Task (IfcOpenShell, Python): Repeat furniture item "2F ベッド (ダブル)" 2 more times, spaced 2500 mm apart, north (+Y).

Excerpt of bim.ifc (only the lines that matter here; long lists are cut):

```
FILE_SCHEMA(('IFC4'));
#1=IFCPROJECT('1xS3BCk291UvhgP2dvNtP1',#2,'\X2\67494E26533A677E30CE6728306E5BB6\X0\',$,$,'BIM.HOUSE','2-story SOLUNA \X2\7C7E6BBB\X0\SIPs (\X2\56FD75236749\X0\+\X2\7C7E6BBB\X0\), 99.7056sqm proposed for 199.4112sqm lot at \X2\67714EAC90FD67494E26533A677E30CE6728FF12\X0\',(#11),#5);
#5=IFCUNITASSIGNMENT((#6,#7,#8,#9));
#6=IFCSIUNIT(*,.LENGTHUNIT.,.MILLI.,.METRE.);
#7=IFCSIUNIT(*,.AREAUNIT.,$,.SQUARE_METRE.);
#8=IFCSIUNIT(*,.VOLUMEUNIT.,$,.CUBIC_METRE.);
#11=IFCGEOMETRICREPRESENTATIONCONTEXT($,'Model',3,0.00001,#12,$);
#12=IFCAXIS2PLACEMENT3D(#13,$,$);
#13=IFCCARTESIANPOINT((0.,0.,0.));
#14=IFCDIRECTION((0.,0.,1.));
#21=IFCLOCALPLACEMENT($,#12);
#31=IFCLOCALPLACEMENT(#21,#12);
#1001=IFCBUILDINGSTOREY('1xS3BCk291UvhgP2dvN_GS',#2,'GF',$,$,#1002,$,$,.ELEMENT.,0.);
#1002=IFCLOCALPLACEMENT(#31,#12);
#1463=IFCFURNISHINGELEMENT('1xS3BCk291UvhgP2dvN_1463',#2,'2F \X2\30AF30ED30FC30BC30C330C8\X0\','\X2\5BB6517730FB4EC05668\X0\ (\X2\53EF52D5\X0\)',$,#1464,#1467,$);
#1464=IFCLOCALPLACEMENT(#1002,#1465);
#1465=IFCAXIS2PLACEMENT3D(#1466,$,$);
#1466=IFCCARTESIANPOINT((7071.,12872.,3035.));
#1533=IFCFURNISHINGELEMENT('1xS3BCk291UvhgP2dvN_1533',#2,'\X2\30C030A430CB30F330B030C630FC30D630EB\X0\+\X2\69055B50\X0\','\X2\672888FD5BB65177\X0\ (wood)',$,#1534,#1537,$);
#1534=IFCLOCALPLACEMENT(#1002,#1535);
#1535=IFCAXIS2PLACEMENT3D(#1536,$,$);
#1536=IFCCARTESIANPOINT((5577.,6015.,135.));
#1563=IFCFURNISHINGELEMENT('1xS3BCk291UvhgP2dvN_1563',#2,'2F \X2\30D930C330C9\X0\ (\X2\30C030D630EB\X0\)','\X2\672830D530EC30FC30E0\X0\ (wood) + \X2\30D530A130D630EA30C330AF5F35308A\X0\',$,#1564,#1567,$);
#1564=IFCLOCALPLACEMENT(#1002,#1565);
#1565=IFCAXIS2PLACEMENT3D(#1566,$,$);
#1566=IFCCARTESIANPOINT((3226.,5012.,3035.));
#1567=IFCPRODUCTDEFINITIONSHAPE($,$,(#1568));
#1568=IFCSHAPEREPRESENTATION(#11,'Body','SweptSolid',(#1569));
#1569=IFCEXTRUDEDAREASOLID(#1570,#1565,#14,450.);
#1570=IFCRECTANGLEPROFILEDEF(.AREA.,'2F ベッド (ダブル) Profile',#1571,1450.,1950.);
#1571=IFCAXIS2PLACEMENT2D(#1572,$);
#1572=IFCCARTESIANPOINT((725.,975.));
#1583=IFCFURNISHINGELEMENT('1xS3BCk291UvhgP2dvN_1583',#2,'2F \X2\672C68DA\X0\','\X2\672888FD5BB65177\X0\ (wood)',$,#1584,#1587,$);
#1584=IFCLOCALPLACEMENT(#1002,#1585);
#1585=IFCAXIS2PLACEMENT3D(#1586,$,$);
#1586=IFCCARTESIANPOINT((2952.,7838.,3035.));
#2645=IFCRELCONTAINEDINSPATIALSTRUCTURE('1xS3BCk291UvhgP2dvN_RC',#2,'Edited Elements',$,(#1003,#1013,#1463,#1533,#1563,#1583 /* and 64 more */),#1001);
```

```python
import numpy as np
import ifcopenshell
import ifcopenshell.api.geometry
import ifcopenshell.api.root
import ifcopenshell.util.element
import ifcopenshell.util.placement

model = ifcopenshell.open("bim.ifc")


def reuse_history(source, copy):
    """copy_class also copies each property set's owner history, people and application; keep the originals."""
    for rel in copy.IsDefinedBy:
        if rel.is_a("IfcRelDefinesByProperties") and (history := rel.RelatingPropertyDefinition.OwnerHistory):
            rel.RelatingPropertyDefinition.OwnerHistory = source.OwnerHistory
            ifcopenshell.util.element.remove_deep2(model, history)


source = model.by_guid("1xS3BCk291UvhgP2dvN_1563")
base = ifcopenshell.util.placement.get_local_placement(source.ObjectPlacement)
step = np.array([0.0, 1.0, 0.0]) * 2500.0

for i in range(1, 3):
    copy = ifcopenshell.api.root.copy_class(model, product=source)
    copy.Representation = ifcopenshell.util.element.copy_deep(
        model, source.Representation, exclude=["IfcGeometricRepresentationContext", "IfcRepresentationMap"]
    )
    reuse_history(source, copy)
    matrix = base.copy()
    matrix[:3, 3] += i * step
    print("added at", matrix[:3, 3].round(3) + 0.0)
    ifcopenshell.api.geometry.edit_object_placement(model, product=copy, matrix=matrix, is_si=False)

model.write("bim_edited.ifc")
```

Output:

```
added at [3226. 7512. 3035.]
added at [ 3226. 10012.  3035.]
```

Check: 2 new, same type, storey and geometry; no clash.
